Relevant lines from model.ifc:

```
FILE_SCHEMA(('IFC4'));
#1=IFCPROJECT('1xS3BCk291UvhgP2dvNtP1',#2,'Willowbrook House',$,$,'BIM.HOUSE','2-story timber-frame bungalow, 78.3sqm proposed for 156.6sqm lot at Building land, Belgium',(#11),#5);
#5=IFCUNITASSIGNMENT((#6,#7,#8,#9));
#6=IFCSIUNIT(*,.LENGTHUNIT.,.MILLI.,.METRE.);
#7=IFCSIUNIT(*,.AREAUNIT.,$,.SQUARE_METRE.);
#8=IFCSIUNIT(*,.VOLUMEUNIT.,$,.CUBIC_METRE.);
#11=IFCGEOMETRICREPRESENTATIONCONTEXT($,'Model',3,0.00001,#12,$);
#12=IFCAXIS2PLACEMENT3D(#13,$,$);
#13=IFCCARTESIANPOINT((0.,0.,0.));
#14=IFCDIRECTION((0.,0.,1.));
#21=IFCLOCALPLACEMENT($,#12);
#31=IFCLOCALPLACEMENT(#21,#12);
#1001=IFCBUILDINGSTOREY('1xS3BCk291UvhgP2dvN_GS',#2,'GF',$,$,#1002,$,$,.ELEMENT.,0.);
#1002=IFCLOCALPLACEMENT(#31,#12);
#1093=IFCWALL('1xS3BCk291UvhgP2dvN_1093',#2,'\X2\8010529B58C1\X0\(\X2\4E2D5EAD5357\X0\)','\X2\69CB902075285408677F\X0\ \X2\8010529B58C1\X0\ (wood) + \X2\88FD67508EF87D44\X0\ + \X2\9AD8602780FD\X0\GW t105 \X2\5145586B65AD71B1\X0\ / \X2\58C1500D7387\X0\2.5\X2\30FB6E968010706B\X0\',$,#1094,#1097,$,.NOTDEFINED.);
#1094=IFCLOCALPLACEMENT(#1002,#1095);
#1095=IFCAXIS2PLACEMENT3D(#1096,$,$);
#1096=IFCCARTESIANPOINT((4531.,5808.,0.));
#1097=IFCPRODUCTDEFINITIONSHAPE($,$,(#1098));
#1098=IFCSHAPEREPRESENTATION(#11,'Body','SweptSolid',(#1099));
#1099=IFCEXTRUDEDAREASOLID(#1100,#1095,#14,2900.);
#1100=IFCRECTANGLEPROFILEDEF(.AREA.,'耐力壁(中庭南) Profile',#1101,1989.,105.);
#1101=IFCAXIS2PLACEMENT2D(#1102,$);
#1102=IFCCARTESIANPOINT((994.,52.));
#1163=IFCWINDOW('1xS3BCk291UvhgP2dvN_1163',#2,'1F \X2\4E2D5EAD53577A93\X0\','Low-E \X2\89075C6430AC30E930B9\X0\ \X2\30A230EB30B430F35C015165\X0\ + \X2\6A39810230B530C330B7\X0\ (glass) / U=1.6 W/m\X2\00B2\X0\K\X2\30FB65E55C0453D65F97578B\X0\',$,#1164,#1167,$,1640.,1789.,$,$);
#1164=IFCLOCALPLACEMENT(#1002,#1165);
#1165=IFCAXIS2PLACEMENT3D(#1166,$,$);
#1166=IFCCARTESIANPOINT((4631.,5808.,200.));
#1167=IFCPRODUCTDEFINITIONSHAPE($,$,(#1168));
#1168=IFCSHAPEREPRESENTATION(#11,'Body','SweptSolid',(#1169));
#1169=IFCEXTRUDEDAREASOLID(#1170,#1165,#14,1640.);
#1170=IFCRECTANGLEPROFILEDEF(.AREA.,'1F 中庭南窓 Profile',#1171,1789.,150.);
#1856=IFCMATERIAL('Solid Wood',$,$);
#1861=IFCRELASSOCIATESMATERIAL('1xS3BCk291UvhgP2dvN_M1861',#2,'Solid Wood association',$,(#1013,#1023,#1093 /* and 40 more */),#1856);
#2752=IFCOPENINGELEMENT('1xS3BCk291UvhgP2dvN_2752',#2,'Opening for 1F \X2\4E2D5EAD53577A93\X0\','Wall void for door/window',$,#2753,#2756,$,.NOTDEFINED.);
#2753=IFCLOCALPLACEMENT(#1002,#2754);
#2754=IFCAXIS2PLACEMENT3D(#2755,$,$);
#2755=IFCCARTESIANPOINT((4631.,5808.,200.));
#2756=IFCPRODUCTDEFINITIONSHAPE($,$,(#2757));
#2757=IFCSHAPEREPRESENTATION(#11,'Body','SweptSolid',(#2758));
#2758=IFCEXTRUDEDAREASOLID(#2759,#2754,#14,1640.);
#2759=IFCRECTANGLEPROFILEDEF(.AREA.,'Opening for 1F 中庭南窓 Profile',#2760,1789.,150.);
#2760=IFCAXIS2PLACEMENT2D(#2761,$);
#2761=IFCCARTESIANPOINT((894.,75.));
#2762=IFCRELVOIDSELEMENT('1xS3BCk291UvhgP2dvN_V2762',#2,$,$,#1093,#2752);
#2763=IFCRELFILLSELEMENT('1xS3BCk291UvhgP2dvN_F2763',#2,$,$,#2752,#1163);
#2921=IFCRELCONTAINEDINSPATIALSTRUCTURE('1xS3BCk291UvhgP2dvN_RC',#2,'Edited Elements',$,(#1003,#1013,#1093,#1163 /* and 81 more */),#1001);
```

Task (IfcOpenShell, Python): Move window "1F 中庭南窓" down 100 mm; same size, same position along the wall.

```python
import numpy as np
import ifcopenshell
import ifcopenshell.api.geometry
import ifcopenshell.util.placement
import ifcopenshell.util.unit

model = ifcopenshell.open("model.ifc")
unit_scale = ifcopenshell.util.unit.calculate_unit_scale(model)

window = model.by_id(1163)
opening = window.FillsVoids[0].RelatingOpeningElement
dz = -100.0

shift = np.array([0.0, 0.0, dz])
# The window is not placed relative to its opening, so move both.
for product in (opening, window):
    matrix = ifcopenshell.util.placement.get_local_placement(product.ObjectPlacement)
    matrix[:3, 3] += shift
    ifcopenshell.api.geometry.edit_object_placement(model, product=product, matrix=matrix, is_si=False)

print(f"moved by {dz * unit_scale:+.3f} m")

model.write("model_rev.ifc")
```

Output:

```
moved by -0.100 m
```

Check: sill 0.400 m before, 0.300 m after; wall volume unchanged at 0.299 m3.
